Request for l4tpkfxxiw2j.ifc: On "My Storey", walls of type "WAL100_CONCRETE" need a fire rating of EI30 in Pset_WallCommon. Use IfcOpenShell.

First a look at what the model holds.

```python
import ifcopenshell
import ifcopenshell.util.element

model = ifcopenshell.open("l4tpkfxxiw2j.ifc")
print(model.schema)
storey = next(s for s in model.by_type("IfcBuildingStorey") if s.Name == "My Storey")
walls = [e for e in ifcopenshell.util.element.get_decomposition(storey) if e.is_a("IfcWall")]
seen = {}
for e in walls:
    element_type = ifcopenshell.util.element.get_type(e)
    key = (element_type.Name if element_type != e and element_type else None, ifcopenshell.util.element.get_pset(e, "Pset_WallCommon", "FireRating"))
    seen[key] = seen.get(key, 0) + 1
for (name, value), count in sorted(seen.items(), key=str):
    print(count, "x", name, "|", value)
```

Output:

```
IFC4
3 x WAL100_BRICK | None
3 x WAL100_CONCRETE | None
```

```python
import ifcopenshell
import ifcopenshell.api.pset
import ifcopenshell.util.element

model = ifcopenshell.open("l4tpkfxxiw2j.ifc")

storey = next(s for s in model.by_type("IfcBuildingStorey") if s.Name == "My Storey")
walls = [e for e in ifcopenshell.util.element.get_decomposition(storey) if e.is_a("IfcWall")]

count = 0
for e in walls:
    element_type = ifcopenshell.util.element.get_type(e)
    if element_type in (None, e) or element_type.Name != "WAL100_CONCRETE":
        continue
    # add_pset returns the element's existing set when there is one.
    pset = ifcopenshell.api.pset.add_pset(model, product=e, name="Pset_WallCommon")
    ifcopenshell.api.pset.edit_pset(model, pset=pset, properties={"FireRating": "EI30"})
    count += 1

print(count, "walls updated")

model.write("l4tpkfxxiw2j_updated.ifc")
```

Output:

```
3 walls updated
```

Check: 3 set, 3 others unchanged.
